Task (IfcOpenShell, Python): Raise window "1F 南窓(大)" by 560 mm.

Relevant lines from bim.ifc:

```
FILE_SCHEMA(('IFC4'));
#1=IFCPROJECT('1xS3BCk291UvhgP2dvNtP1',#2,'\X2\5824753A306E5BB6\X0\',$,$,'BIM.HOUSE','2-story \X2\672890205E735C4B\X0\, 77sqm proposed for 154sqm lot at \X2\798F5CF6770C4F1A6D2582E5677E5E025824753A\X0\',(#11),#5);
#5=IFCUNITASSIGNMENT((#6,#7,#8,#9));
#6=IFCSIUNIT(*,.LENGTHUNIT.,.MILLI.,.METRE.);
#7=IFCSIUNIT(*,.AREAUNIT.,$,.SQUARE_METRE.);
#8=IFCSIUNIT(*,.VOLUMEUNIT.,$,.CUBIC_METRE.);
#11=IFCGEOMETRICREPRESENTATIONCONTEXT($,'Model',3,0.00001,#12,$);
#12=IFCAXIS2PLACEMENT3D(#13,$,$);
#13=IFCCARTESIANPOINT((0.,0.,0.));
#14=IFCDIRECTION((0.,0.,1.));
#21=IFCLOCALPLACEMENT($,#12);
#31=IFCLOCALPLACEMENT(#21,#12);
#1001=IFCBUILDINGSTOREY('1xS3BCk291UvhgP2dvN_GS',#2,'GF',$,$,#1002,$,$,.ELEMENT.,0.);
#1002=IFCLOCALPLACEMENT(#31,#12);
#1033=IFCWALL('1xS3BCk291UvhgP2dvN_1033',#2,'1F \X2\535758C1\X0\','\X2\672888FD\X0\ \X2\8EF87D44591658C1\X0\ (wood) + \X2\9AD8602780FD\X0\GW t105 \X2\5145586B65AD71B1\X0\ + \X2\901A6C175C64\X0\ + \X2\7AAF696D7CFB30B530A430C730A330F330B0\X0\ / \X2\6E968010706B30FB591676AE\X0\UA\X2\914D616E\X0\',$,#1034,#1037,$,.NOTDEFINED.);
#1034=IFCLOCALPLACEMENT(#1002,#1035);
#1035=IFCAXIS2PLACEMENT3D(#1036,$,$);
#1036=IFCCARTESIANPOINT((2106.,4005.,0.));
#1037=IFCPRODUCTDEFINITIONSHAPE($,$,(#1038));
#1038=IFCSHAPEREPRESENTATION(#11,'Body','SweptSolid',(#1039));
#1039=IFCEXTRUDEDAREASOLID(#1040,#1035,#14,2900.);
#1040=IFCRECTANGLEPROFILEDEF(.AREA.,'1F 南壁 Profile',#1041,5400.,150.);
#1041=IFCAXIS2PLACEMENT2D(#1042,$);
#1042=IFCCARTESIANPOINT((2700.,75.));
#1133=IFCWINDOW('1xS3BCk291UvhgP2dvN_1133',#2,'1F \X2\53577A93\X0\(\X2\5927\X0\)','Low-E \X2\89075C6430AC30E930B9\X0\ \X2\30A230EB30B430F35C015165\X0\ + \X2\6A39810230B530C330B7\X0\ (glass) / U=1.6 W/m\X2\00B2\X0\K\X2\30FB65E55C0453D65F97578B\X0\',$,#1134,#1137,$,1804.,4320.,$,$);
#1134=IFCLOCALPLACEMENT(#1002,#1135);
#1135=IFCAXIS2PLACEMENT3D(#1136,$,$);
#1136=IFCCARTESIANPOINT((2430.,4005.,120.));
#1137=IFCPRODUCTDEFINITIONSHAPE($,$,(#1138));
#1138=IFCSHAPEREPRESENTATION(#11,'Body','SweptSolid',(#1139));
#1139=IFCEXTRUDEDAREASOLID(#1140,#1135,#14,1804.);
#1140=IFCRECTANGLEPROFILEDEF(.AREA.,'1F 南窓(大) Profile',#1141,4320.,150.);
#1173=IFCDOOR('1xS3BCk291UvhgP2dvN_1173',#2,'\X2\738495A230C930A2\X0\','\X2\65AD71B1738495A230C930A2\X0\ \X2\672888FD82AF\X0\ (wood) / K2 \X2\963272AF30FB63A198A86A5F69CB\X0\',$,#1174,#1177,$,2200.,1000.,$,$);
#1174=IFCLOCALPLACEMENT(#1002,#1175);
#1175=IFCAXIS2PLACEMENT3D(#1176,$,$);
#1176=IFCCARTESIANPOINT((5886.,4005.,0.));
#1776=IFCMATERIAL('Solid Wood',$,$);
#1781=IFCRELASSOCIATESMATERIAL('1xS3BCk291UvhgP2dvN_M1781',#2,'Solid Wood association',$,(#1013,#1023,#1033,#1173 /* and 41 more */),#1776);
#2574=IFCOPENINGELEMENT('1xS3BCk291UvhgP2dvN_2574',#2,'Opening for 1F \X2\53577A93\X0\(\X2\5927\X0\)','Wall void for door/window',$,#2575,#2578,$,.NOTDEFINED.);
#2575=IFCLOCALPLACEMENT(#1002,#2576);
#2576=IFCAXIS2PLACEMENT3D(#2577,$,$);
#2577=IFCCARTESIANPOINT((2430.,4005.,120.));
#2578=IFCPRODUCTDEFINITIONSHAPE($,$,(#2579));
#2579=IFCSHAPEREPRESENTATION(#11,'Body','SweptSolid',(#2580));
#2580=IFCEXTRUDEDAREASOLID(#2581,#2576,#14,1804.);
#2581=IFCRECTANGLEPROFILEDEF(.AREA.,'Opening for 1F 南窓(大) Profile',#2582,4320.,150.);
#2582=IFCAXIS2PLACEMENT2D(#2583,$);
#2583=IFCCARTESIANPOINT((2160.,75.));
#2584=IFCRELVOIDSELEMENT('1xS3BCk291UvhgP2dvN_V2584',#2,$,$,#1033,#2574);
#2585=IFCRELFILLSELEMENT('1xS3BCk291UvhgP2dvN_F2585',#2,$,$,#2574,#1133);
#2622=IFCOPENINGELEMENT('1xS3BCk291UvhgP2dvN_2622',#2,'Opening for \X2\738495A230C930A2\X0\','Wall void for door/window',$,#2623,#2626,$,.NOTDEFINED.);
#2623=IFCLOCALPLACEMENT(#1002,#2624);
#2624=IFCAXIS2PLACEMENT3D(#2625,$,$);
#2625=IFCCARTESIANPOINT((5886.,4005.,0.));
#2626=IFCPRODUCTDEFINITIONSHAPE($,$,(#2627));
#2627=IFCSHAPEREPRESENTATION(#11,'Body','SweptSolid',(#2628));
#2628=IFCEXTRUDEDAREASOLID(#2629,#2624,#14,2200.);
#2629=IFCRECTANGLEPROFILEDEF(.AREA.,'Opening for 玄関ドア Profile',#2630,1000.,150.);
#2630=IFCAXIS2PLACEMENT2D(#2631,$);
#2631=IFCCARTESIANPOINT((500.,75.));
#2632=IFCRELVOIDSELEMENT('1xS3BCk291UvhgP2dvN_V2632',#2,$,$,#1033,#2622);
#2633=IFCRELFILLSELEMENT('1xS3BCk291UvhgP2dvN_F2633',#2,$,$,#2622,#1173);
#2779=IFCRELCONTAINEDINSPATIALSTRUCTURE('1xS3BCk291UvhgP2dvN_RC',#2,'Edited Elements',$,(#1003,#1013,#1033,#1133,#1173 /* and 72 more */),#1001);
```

```python
import numpy as np
import ifcopenshell
import ifcopenshell.api.geometry
import ifcopenshell.util.placement
import ifcopenshell.util.unit

model = ifcopenshell.open("bim.ifc")
unit_scale = ifcopenshell.util.unit.calculate_unit_scale(model)

window = model.by_guid("1xS3BCk291UvhgP2dvN_1133")
opening = window.FillsVoids[0].RelatingOpeningElement
dz = 560.0

shift = np.array([0.0, 0.0, dz])
# The window is not placed relative to its opening, so move both.
for product in (opening, window):
    matrix = ifcopenshell.util.placement.get_local_placement(product.ObjectPlacement)
    matrix[:3, 3] += shift
    ifcopenshell.api.geometry.edit_object_placement(model, product=product, matrix=matrix, is_si=False)

print(f"moved by {dz * unit_scale:+.3f} m")

model.write("bim-out.ifc")
```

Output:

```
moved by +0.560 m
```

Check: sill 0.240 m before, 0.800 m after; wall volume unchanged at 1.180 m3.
